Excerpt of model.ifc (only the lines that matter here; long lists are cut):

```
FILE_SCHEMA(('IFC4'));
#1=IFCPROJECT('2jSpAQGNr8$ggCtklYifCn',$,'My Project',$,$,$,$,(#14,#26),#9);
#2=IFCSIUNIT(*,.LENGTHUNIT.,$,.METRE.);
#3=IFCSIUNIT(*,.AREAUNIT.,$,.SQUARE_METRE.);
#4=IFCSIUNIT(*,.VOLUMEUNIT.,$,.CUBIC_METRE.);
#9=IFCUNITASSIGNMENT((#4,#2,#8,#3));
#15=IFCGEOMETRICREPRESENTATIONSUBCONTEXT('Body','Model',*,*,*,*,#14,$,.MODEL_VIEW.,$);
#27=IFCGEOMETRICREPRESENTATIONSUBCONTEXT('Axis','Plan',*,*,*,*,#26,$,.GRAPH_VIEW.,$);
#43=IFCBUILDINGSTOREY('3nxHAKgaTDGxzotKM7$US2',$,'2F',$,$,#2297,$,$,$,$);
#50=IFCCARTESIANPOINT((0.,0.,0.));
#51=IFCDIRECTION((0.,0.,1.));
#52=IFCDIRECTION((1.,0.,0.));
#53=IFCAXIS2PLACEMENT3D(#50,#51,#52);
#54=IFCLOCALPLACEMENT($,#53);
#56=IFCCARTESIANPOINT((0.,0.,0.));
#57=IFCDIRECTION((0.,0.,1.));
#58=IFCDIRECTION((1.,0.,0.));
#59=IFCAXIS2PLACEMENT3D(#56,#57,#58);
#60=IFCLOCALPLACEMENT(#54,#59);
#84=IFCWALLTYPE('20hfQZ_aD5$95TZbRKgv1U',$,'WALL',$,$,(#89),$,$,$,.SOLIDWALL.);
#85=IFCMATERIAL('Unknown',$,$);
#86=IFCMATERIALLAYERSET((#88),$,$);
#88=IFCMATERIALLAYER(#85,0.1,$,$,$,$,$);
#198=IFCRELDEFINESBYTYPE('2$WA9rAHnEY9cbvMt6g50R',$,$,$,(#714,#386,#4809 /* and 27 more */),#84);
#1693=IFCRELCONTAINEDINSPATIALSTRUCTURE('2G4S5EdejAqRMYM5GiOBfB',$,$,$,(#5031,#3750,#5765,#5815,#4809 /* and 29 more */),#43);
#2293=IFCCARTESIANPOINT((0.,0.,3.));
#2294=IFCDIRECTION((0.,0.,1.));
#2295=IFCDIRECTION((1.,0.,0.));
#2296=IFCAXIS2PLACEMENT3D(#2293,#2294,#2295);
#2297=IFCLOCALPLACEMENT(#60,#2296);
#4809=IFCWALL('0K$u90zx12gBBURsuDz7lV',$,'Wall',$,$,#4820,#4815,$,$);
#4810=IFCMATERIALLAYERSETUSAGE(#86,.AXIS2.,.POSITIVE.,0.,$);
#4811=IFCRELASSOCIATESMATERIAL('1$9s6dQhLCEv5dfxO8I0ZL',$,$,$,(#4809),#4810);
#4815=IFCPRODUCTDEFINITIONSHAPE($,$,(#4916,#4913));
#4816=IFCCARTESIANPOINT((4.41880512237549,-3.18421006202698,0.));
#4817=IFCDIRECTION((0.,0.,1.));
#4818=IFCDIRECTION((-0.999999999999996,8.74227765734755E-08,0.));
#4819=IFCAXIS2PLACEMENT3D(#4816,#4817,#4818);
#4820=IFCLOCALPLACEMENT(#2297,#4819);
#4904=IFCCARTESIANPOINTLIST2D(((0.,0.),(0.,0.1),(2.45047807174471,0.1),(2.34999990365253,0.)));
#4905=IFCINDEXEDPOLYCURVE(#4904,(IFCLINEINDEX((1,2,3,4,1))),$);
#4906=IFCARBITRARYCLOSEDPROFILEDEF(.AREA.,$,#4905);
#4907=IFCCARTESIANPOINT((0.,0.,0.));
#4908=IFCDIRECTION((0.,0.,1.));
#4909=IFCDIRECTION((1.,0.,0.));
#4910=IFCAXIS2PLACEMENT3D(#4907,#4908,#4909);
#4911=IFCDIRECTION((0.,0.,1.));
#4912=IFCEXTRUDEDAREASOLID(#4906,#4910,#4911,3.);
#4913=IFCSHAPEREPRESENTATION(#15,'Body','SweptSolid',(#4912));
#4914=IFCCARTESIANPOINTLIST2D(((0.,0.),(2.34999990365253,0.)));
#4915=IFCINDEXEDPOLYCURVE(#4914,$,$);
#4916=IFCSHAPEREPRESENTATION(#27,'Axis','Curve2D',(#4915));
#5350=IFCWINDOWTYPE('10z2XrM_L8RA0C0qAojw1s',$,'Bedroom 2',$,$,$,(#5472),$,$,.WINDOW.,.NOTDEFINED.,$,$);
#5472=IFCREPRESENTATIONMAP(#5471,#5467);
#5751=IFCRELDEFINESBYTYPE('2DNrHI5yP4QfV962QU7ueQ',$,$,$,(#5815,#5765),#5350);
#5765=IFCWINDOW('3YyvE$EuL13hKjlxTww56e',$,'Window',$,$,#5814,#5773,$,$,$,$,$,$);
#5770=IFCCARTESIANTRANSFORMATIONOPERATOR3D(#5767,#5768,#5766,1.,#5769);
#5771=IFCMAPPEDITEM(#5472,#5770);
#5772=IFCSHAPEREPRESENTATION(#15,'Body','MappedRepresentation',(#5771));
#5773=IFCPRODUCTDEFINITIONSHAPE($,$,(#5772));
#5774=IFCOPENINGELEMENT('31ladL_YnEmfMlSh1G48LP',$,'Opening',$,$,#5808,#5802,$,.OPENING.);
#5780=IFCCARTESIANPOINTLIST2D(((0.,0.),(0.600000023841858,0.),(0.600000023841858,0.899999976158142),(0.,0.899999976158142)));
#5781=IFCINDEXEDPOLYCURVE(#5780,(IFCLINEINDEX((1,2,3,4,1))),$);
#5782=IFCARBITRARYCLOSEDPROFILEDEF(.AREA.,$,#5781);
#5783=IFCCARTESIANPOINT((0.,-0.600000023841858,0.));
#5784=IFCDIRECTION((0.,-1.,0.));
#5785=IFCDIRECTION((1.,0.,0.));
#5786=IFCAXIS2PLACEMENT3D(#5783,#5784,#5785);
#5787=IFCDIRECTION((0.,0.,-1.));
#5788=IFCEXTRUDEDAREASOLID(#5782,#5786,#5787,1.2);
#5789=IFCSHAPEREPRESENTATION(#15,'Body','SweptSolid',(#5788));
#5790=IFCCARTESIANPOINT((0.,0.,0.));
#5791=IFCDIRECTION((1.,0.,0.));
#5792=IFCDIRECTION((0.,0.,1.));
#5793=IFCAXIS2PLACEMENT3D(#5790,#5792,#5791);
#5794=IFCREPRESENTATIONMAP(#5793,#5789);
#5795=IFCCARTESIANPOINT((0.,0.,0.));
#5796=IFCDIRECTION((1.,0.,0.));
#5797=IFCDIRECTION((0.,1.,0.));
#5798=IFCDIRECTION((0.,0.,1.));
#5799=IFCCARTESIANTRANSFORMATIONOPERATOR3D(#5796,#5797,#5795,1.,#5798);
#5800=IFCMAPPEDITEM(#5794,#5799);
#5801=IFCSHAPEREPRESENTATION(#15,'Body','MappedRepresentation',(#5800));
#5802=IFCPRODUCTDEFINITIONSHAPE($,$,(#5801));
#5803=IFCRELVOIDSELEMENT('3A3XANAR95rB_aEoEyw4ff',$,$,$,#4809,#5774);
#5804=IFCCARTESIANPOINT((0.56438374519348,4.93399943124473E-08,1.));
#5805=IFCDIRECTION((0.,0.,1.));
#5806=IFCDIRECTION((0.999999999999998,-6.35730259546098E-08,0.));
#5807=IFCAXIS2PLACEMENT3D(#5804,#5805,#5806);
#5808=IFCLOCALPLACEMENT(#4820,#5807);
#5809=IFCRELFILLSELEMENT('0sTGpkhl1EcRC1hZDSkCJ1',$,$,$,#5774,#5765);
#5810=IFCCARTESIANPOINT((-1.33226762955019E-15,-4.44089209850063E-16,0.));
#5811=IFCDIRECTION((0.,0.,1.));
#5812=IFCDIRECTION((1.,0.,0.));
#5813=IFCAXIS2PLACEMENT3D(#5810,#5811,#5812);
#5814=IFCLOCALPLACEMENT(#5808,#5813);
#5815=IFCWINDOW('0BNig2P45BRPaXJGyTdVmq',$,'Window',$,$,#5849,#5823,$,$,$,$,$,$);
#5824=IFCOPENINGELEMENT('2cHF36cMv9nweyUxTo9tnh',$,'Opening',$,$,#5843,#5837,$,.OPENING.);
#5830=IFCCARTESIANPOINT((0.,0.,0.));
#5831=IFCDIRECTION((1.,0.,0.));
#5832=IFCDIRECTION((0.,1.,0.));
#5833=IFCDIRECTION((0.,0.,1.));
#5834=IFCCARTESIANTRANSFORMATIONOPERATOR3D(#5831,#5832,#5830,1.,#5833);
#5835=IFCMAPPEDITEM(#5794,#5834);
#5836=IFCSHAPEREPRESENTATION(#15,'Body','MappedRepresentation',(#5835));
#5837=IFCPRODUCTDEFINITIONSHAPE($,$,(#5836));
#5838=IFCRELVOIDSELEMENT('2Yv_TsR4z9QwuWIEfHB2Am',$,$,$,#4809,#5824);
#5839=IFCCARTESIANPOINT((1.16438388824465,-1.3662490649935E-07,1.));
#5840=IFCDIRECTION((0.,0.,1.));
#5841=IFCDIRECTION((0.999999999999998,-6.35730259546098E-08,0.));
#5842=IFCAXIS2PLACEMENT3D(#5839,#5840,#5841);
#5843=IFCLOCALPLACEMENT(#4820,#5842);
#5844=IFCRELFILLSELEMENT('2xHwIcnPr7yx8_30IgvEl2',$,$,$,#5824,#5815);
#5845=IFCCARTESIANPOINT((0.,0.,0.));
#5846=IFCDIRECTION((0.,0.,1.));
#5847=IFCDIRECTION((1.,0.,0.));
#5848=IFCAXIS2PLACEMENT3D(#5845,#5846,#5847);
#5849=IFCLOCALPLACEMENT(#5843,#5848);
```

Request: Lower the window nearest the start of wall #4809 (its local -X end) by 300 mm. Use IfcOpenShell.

```python
import numpy as np
import ifcopenshell
import ifcopenshell.api.geometry
import ifcopenshell.util.placement
import ifcopenshell.util.unit

model = ifcopenshell.open("model.ifc")
unit_scale = ifcopenshell.util.unit.calculate_unit_scale(model)

window = model.by_guid("3YyvE$EuL13hKjlxTww56e")
opening = window.FillsVoids[0].RelatingOpeningElement
dz = -0.3

shift = np.array([0.0, 0.0, dz])
# The window is placed relative to its opening, so it follows when the opening moves.
matrix = ifcopenshell.util.placement.get_local_placement(opening.ObjectPlacement)
matrix[:3, 3] += shift
ifcopenshell.api.geometry.edit_object_placement(
    model, product=opening, matrix=matrix, is_si=False, should_transform_children=True
)

print(f"moved by {dz * unit_scale:+.3f} m")

model.write("model_v2.ifc")
```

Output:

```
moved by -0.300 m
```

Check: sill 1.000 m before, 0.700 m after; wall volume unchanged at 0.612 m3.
